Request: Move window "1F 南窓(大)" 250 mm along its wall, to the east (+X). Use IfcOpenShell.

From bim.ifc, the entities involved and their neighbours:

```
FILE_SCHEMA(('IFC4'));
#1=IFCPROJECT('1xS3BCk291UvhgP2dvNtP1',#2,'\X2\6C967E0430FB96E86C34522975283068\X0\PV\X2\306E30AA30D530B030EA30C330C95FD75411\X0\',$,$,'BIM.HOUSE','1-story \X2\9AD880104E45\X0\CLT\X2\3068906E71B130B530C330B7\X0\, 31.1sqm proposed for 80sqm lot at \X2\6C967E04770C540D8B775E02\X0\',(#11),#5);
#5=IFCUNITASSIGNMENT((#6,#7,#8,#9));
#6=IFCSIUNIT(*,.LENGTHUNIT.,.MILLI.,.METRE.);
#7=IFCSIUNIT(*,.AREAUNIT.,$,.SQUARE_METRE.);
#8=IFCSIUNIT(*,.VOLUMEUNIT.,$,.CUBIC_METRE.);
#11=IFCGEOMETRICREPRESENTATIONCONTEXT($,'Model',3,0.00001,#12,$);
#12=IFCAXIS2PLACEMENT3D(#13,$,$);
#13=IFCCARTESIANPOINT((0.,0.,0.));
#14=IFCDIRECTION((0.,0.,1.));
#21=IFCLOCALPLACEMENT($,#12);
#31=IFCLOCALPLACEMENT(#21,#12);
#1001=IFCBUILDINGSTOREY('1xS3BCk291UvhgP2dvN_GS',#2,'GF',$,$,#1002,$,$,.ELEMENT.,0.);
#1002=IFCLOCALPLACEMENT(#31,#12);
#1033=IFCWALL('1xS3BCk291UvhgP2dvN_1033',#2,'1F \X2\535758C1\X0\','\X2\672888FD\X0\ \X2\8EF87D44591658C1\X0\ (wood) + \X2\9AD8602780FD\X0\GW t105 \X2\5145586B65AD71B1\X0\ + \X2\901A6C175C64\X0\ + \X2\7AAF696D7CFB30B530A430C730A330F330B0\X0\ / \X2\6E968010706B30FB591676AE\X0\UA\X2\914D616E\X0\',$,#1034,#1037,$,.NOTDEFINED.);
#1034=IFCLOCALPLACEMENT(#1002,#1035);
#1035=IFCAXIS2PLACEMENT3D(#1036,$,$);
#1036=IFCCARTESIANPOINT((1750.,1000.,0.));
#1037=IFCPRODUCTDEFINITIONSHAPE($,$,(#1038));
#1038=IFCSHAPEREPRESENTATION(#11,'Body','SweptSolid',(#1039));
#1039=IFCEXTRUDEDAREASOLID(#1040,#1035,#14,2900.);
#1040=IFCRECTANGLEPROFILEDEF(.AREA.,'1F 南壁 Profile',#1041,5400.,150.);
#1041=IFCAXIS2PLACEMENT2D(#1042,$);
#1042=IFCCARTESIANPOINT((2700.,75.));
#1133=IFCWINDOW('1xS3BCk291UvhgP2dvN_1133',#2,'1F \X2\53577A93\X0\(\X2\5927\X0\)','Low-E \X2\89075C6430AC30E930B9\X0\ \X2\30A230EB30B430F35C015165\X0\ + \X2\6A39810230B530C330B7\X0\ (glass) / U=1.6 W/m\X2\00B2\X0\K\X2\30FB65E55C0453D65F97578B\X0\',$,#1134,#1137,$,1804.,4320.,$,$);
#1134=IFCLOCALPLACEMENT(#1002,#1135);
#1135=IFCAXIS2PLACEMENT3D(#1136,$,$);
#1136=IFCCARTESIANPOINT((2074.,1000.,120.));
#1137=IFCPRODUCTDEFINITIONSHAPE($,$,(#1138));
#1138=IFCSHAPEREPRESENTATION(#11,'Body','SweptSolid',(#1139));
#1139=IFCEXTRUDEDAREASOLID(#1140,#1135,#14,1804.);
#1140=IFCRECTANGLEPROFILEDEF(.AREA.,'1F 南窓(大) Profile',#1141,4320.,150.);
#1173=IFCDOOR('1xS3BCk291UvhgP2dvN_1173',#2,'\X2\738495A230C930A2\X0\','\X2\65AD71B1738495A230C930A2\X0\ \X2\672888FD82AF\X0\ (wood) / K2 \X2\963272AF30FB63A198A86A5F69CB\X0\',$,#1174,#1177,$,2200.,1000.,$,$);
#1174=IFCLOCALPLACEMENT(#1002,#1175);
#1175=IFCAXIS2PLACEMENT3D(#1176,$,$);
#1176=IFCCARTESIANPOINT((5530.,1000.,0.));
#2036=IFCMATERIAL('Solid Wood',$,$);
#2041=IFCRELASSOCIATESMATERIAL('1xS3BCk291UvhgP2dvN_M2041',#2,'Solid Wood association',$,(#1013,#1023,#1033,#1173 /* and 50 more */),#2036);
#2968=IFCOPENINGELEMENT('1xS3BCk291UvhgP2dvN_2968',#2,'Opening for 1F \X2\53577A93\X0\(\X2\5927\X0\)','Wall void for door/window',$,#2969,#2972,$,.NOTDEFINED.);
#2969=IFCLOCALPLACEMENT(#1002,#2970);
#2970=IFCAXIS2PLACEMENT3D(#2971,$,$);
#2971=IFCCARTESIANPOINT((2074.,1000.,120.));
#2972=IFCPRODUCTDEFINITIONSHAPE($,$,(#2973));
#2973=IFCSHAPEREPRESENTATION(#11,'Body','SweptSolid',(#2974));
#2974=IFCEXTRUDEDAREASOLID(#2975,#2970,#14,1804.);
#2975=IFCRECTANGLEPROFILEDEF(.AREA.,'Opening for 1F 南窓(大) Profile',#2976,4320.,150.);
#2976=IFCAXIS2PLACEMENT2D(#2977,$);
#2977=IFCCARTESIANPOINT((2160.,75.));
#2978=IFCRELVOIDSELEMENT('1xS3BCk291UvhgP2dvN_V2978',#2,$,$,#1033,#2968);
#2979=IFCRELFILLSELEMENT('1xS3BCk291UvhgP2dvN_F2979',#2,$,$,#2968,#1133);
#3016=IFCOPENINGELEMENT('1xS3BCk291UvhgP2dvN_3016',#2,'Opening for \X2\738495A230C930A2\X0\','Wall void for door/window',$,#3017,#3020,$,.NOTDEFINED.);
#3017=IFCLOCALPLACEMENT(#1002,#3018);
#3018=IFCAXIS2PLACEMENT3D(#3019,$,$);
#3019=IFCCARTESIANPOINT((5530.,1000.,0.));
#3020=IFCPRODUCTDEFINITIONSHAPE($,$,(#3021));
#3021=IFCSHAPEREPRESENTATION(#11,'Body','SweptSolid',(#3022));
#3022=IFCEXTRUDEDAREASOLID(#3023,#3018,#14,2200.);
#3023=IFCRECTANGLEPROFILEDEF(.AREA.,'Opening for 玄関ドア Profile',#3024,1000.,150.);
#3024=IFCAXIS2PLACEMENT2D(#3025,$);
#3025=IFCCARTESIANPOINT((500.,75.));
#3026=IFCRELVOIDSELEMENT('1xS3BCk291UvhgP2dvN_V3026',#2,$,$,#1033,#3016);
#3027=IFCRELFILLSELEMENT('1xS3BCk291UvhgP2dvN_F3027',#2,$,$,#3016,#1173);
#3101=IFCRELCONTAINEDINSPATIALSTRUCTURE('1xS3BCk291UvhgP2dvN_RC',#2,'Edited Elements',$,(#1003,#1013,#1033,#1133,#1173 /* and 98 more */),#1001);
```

```python
import ifcopenshell
import ifcopenshell.api.geometry
import ifcopenshell.util.placement

model = ifcopenshell.open("bim.ifc")

window = model.by_guid("1xS3BCk291UvhgP2dvN_1133")
opening = window.FillsVoids[0].RelatingOpeningElement
wall = opening.VoidsElements[0].RelatingBuildingElement

wall_matrix = ifcopenshell.util.placement.get_local_placement(wall.ObjectPlacement)
shift = wall_matrix[:3, 0] * 250.0
before = ifcopenshell.util.placement.get_local_placement(window.ObjectPlacement)[:3, 3].copy()

# The window is not placed relative to its opening, so move both.
for product in (opening, window):
    matrix = ifcopenshell.util.placement.get_local_placement(product.ObjectPlacement)
    matrix[:3, 3] += shift
    ifcopenshell.api.geometry.edit_object_placement(model, product=product, matrix=matrix, is_si=False)

after = ifcopenshell.util.placement.get_local_placement(window.ObjectPlacement)[:3, 3]
print("window moved by", (after - before).round(3) + 0.0)

model.write("bim-out.ifc")
```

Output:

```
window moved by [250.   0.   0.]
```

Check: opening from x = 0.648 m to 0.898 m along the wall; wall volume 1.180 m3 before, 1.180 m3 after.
